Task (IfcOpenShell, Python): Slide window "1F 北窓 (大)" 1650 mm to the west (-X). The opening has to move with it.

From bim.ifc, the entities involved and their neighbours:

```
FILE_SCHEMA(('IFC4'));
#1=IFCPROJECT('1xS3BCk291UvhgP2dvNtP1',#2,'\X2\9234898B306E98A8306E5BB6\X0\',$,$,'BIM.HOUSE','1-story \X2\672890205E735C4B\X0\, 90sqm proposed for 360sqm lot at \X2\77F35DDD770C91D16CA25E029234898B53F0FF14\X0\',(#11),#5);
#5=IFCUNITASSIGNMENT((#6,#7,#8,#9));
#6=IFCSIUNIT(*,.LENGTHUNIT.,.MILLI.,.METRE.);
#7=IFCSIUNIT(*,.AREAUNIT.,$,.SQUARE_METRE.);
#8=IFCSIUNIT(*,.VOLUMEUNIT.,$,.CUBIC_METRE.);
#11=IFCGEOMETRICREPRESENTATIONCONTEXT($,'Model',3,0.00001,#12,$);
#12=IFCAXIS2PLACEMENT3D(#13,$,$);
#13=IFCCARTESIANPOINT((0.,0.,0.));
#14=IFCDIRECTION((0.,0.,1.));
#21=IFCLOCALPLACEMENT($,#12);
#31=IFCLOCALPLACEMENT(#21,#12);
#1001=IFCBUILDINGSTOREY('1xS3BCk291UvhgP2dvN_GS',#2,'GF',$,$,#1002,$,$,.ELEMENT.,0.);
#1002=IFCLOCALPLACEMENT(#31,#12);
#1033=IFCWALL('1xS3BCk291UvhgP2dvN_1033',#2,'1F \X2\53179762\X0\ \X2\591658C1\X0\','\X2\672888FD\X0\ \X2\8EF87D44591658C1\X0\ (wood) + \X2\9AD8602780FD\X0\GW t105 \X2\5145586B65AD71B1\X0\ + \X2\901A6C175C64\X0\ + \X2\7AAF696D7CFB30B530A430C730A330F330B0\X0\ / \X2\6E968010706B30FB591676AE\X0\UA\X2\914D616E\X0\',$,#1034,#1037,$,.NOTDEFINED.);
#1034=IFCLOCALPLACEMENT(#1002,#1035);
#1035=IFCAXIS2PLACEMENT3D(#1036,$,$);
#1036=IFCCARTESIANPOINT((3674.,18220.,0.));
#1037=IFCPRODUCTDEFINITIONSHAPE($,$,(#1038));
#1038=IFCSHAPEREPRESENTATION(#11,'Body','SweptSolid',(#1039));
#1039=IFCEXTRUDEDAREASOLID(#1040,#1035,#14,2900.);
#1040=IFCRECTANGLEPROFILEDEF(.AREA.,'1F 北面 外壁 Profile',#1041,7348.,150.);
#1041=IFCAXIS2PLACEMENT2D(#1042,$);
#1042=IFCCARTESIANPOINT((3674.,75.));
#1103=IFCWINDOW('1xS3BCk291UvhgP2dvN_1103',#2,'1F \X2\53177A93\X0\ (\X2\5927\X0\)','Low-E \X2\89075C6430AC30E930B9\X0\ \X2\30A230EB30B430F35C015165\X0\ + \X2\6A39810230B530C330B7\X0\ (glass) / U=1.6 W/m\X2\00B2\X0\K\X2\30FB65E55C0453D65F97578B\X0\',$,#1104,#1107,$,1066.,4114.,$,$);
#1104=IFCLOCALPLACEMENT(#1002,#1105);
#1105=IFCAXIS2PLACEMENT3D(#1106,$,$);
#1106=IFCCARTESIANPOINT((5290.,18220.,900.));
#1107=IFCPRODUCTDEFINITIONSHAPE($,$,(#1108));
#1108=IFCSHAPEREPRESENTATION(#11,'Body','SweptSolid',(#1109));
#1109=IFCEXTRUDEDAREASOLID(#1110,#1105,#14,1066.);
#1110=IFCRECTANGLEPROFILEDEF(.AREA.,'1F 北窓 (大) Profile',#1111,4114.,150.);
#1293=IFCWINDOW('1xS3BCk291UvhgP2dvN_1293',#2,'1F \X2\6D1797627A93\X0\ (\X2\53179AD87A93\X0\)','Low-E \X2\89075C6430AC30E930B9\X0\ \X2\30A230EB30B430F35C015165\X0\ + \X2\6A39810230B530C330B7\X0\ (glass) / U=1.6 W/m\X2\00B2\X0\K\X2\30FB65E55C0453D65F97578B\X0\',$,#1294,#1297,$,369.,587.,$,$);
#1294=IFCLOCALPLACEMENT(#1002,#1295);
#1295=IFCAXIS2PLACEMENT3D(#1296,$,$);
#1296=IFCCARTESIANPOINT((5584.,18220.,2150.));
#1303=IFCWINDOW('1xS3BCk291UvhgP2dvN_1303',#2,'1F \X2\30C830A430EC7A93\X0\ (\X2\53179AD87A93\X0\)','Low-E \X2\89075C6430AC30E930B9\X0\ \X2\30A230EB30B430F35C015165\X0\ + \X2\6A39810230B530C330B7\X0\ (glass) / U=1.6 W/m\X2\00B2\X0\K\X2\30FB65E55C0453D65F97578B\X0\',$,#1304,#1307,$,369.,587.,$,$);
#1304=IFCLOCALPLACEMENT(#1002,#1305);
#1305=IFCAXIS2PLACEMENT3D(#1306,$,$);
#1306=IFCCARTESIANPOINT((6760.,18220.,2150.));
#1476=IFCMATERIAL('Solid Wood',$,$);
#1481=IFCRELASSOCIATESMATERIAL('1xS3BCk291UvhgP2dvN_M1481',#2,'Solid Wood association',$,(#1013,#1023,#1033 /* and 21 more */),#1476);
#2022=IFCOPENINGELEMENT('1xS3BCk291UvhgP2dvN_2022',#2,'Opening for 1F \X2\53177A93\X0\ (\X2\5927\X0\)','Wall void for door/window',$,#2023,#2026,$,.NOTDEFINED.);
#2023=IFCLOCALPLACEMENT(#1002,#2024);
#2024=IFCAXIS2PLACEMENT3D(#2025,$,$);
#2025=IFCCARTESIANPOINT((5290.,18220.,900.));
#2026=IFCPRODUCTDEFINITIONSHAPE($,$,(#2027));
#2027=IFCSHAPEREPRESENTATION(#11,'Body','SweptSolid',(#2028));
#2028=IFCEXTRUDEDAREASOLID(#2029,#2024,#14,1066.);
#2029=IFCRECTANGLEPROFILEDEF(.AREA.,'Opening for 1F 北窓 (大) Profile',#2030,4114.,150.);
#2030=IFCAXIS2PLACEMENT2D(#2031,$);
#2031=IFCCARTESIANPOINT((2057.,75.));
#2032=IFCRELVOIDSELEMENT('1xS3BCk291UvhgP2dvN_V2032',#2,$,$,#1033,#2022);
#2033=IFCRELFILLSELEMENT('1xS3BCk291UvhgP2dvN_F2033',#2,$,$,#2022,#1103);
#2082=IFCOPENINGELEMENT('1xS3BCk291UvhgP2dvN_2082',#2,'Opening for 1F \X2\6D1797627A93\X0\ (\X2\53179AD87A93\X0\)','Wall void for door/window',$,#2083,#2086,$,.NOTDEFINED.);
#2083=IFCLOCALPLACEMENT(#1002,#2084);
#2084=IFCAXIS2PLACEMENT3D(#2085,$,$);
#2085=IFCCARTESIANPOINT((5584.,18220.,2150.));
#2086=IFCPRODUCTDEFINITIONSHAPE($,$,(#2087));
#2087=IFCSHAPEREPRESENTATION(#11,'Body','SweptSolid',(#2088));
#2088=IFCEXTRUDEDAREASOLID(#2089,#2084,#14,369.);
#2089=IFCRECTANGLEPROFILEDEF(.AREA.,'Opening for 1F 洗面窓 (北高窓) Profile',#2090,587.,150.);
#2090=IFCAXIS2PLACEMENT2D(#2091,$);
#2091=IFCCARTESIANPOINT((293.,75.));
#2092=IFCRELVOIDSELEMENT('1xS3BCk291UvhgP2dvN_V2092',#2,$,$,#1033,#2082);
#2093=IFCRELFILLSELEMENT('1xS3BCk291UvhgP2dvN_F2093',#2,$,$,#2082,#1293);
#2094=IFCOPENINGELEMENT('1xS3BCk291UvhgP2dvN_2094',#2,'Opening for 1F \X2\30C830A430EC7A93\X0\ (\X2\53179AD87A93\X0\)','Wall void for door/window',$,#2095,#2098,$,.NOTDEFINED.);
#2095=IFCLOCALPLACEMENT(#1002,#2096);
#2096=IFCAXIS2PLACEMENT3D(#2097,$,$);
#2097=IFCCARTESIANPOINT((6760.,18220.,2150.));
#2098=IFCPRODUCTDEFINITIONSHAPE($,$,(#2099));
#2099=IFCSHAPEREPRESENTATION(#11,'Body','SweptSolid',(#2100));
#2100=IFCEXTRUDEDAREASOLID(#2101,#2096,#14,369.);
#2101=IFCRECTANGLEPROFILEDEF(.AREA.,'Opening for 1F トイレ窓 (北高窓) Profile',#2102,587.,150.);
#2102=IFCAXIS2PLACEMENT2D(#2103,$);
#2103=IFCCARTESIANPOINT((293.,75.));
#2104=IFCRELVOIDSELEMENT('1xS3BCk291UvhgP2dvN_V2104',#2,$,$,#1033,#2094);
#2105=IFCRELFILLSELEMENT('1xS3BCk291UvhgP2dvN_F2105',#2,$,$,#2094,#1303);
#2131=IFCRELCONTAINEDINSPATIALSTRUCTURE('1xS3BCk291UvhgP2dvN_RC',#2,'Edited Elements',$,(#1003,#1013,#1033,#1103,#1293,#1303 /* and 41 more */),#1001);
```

```python
import ifcopenshell
import ifcopenshell.api.geometry
import ifcopenshell.util.placement
import ifcopenshell.util.unit

model = ifcopenshell.open("bim.ifc")
unit_scale = ifcopenshell.util.unit.calculate_unit_scale(model)

window = model.by_guid("1xS3BCk291UvhgP2dvN_1103")
opening = window.FillsVoids[0].RelatingOpeningElement
wall = opening.VoidsElements[0].RelatingBuildingElement

wall_matrix = ifcopenshell.util.placement.get_local_placement(wall.ObjectPlacement)
shift = wall_matrix[:3, 0] * -1.65 / unit_scale
before = ifcopenshell.util.placement.get_local_placement(window.ObjectPlacement)[:3, 3].copy()

# The window is not placed relative to its opening, so move both.
for product in (opening, window):
    matrix = ifcopenshell.util.placement.get_local_placement(product.ObjectPlacement)
    matrix[:3, 3] += shift
    ifcopenshell.api.geometry.edit_object_placement(model, product=product, matrix=matrix, is_si=False)

after = ifcopenshell.util.placement.get_local_placement(window.ObjectPlacement)[:3, 3]
print("window moved by", (after - before).round(3) + 0.0)

model.write("bim_rev.ifc")
```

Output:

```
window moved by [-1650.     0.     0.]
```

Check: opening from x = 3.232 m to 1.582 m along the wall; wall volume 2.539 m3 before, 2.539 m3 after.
